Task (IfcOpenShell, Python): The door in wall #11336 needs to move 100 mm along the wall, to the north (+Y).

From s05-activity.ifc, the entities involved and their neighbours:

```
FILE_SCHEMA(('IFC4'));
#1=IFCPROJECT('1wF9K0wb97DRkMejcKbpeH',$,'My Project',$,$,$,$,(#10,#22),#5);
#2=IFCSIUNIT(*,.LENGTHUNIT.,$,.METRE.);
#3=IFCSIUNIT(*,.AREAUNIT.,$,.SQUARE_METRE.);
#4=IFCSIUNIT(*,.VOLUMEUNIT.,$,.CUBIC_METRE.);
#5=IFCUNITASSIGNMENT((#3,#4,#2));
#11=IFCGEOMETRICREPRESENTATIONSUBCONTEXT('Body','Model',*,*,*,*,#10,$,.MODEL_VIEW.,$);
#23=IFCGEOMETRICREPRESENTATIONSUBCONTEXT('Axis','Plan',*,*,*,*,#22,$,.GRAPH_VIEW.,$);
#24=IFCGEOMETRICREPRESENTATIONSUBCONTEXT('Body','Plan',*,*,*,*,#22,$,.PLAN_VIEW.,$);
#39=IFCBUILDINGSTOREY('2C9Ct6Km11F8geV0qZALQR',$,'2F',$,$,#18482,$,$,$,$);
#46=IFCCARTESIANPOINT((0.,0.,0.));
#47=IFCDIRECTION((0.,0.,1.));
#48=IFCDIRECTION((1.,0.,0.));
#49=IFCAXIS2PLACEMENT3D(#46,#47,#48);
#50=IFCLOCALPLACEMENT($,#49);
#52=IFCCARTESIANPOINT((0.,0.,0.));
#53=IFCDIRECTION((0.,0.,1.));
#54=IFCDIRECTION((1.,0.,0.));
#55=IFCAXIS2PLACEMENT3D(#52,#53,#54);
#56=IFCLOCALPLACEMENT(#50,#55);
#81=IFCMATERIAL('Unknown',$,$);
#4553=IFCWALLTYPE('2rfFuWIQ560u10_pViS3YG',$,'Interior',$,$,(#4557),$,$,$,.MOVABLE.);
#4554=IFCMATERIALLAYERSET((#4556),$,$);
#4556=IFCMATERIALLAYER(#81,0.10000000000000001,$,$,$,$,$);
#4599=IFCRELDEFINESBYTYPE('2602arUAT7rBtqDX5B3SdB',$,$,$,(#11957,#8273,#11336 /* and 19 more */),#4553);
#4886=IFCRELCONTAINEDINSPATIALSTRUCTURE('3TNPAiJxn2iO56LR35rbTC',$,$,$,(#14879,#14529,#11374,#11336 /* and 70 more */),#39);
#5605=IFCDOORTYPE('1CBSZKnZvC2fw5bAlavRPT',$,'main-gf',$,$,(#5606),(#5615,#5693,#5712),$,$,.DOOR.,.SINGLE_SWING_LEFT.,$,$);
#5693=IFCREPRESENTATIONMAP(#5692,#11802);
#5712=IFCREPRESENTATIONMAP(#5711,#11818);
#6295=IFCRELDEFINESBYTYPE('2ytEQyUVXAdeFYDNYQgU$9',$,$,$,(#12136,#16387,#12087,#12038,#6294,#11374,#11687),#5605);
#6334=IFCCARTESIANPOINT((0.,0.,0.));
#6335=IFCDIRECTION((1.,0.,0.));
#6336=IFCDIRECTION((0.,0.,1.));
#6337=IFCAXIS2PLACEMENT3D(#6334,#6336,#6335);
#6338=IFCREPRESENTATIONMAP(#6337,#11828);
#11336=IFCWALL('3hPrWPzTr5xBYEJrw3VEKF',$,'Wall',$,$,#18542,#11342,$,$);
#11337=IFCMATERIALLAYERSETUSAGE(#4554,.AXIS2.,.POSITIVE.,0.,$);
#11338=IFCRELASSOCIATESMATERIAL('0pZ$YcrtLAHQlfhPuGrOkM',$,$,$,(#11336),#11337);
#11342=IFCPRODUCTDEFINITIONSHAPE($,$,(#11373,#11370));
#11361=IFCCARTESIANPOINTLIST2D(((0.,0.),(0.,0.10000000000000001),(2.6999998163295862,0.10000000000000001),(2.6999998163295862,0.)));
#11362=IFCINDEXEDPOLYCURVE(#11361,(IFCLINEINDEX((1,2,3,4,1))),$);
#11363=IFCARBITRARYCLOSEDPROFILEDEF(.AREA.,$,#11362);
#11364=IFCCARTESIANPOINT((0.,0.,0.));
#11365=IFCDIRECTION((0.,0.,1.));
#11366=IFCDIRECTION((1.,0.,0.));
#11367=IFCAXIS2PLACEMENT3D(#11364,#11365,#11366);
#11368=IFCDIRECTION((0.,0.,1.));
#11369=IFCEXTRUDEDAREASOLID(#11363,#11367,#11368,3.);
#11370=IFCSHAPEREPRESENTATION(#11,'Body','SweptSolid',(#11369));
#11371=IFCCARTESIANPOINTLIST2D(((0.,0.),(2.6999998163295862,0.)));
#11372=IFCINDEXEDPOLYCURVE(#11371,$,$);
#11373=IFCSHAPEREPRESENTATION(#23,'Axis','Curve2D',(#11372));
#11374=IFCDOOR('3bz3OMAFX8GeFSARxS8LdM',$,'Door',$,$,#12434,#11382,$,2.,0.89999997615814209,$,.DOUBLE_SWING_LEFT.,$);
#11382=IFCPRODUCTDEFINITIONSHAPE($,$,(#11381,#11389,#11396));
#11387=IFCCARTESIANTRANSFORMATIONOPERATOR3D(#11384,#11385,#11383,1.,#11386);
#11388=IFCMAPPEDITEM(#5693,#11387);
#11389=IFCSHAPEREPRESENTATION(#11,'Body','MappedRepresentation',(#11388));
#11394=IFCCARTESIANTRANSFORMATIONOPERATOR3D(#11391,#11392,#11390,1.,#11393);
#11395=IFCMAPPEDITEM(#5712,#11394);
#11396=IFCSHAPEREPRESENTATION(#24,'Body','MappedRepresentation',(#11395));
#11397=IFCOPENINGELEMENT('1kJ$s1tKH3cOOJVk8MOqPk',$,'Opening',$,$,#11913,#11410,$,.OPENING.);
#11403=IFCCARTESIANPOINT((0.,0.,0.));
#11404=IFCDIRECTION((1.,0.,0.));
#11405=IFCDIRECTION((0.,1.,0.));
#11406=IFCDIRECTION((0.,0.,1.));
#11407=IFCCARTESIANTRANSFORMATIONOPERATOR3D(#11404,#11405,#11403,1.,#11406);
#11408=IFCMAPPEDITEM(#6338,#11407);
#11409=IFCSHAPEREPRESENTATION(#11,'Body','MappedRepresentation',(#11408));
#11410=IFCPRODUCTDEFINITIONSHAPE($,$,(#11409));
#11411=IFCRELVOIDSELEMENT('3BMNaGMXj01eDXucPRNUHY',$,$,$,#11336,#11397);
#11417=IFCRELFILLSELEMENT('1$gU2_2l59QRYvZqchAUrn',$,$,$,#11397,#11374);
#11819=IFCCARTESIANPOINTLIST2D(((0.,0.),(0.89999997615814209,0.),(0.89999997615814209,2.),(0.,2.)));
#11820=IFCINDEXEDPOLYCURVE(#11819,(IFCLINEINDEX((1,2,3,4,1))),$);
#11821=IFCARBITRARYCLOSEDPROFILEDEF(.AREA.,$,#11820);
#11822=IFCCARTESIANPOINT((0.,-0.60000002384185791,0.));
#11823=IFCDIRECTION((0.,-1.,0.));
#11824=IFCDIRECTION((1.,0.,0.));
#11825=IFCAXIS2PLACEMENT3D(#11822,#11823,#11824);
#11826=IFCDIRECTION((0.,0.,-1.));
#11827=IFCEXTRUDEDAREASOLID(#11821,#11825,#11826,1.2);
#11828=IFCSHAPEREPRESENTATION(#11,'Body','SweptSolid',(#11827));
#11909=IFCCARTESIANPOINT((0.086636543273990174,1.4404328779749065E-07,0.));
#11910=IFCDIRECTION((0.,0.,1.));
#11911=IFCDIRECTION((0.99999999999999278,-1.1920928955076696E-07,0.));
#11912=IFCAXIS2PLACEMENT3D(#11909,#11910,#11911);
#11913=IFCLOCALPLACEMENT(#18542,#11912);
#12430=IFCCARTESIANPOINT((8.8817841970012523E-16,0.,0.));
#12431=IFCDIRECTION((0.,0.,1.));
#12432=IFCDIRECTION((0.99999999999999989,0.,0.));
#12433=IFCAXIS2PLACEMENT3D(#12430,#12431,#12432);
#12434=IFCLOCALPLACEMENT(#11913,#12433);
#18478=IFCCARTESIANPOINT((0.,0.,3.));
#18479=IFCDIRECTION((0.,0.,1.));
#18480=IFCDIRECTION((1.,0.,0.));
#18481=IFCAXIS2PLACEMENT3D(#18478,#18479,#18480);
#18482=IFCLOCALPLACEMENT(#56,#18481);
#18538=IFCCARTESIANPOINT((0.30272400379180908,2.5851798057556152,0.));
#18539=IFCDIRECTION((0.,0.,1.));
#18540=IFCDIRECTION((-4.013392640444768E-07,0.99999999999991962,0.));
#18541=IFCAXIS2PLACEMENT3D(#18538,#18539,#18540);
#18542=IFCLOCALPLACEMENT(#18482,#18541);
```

```python
import ifcopenshell
import ifcopenshell.api.geometry
import ifcopenshell.util.placement
import ifcopenshell.util.unit

model = ifcopenshell.open("s05-activity.ifc")
unit_scale = ifcopenshell.util.unit.calculate_unit_scale(model)

door = model.by_guid("3bz3OMAFX8GeFSARxS8LdM")
opening = door.FillsVoids[0].RelatingOpeningElement
wall = opening.VoidsElements[0].RelatingBuildingElement

wall_matrix = ifcopenshell.util.placement.get_local_placement(wall.ObjectPlacement)
shift = wall_matrix[:3, 0] * 0.1 / unit_scale
before = ifcopenshell.util.placement.get_local_placement(door.ObjectPlacement)[:3, 3].copy()

# The door is placed relative to its opening, so it follows when the opening moves.
matrix = ifcopenshell.util.placement.get_local_placement(opening.ObjectPlacement)
matrix[:3, 3] += shift
ifcopenshell.api.geometry.edit_object_placement(
    model, product=opening, matrix=matrix, is_si=False, should_transform_children=True
)

after = ifcopenshell.util.placement.get_local_placement(door.ObjectPlacement)[:3, 3]
print("door moved by", (after - before).round(3) + 0.0)

model.write("s05-activity_v2.ifc")
```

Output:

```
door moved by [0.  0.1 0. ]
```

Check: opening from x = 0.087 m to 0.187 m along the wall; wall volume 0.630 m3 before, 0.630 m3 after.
